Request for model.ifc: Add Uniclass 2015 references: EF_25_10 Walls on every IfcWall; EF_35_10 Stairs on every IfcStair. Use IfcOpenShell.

First a look at what the model holds.

```python
import ifcopenshell

model = ifcopenshell.open("model.ifc")
print(model.schema)
print("classifications:", [c.Name for c in model.by_type("IfcClassification")])
for ifc_class in ("IfcDoor", "IfcRoof", "IfcStair", "IfcWall", "IfcWindow"):
    print(ifc_class, len(model.by_type(ifc_class)))
```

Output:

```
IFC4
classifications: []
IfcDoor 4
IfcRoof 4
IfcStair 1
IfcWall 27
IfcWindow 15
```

```python
import ifcopenshell
import ifcopenshell.api.classification

model = ifcopenshell.open("model.ifc")

system = ifcopenshell.api.classification.add_classification(model, classification="Uniclass 2015")

codes = {
    "IfcWall": ("EF_25_10", "Walls"),
    "IfcStair": ("EF_35_10", "Stairs"),
}
for ifc_class, (code, name) in codes.items():
    products = model.by_type(ifc_class)
    ifcopenshell.api.classification.add_reference(
        model, products=products, classification=system, identification=code, name=name
    )
    print(code, len(products))

model.write("model_updated.ifc")
```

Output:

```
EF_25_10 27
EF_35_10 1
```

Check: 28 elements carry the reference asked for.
